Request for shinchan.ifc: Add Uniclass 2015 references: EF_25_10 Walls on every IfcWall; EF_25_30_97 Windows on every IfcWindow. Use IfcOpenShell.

First a look at what the model holds.

```python
import ifcopenshell

model = ifcopenshell.open("shinchan.ifc")
print(model.schema)
print("classifications:", [c.Name for c in model.by_type("IfcClassification")])
for ifc_class in ("IfcDoor", "IfcRoof", "IfcStair", "IfcWall", "IfcWindow"):
    print(ifc_class, len(model.by_type(ifc_class)))
```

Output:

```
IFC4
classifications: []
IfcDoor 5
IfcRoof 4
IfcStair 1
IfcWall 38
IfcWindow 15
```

```python
import ifcopenshell
import ifcopenshell.api.classification

model = ifcopenshell.open("shinchan.ifc")

system = ifcopenshell.api.classification.add_classification(model, classification="Uniclass 2015")

codes = {
    "IfcWall": ("EF_25_10", "Walls"),
    "IfcWindow": ("EF_25_30_97", "Windows"),
}
for ifc_class, (code, name) in codes.items():
    products = model.by_type(ifc_class)
    ifcopenshell.api.classification.add_reference(
        model, products=products, classification=system, identification=code, name=name
    )
    print(code, len(products))

model.write("shinchan_v2.ifc")
```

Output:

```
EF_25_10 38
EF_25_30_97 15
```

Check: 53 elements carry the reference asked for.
